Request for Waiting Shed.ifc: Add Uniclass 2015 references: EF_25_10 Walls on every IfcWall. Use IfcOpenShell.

First a look at what the model holds.

```python
import ifcopenshell

model = ifcopenshell.open("Waiting Shed.ifc")
print(model.schema)
print("classifications:", [c.Name for c in model.by_type("IfcClassification")])
for ifc_class in ("IfcDoor", "IfcRoof", "IfcStair", "IfcWall", "IfcWindow"):
    print(ifc_class, len(model.by_type(ifc_class)))
```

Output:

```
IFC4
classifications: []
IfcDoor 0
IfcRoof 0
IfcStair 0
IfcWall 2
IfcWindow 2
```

```python
import ifcopenshell
import ifcopenshell.api.classification

model = ifcopenshell.open("Waiting Shed.ifc")

system = ifcopenshell.api.classification.add_classification(model, classification="Uniclass 2015")

codes = {
    "IfcWall": ("EF_25_10", "Walls"),
}
for ifc_class, (code, name) in codes.items():
    products = model.by_type(ifc_class)
    ifcopenshell.api.classification.add_reference(
        model, products=products, classification=system, identification=code, name=name
    )
    print(code, len(products))

model.write("Waiting Shed-out.ifc")
```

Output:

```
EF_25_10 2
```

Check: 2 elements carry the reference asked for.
